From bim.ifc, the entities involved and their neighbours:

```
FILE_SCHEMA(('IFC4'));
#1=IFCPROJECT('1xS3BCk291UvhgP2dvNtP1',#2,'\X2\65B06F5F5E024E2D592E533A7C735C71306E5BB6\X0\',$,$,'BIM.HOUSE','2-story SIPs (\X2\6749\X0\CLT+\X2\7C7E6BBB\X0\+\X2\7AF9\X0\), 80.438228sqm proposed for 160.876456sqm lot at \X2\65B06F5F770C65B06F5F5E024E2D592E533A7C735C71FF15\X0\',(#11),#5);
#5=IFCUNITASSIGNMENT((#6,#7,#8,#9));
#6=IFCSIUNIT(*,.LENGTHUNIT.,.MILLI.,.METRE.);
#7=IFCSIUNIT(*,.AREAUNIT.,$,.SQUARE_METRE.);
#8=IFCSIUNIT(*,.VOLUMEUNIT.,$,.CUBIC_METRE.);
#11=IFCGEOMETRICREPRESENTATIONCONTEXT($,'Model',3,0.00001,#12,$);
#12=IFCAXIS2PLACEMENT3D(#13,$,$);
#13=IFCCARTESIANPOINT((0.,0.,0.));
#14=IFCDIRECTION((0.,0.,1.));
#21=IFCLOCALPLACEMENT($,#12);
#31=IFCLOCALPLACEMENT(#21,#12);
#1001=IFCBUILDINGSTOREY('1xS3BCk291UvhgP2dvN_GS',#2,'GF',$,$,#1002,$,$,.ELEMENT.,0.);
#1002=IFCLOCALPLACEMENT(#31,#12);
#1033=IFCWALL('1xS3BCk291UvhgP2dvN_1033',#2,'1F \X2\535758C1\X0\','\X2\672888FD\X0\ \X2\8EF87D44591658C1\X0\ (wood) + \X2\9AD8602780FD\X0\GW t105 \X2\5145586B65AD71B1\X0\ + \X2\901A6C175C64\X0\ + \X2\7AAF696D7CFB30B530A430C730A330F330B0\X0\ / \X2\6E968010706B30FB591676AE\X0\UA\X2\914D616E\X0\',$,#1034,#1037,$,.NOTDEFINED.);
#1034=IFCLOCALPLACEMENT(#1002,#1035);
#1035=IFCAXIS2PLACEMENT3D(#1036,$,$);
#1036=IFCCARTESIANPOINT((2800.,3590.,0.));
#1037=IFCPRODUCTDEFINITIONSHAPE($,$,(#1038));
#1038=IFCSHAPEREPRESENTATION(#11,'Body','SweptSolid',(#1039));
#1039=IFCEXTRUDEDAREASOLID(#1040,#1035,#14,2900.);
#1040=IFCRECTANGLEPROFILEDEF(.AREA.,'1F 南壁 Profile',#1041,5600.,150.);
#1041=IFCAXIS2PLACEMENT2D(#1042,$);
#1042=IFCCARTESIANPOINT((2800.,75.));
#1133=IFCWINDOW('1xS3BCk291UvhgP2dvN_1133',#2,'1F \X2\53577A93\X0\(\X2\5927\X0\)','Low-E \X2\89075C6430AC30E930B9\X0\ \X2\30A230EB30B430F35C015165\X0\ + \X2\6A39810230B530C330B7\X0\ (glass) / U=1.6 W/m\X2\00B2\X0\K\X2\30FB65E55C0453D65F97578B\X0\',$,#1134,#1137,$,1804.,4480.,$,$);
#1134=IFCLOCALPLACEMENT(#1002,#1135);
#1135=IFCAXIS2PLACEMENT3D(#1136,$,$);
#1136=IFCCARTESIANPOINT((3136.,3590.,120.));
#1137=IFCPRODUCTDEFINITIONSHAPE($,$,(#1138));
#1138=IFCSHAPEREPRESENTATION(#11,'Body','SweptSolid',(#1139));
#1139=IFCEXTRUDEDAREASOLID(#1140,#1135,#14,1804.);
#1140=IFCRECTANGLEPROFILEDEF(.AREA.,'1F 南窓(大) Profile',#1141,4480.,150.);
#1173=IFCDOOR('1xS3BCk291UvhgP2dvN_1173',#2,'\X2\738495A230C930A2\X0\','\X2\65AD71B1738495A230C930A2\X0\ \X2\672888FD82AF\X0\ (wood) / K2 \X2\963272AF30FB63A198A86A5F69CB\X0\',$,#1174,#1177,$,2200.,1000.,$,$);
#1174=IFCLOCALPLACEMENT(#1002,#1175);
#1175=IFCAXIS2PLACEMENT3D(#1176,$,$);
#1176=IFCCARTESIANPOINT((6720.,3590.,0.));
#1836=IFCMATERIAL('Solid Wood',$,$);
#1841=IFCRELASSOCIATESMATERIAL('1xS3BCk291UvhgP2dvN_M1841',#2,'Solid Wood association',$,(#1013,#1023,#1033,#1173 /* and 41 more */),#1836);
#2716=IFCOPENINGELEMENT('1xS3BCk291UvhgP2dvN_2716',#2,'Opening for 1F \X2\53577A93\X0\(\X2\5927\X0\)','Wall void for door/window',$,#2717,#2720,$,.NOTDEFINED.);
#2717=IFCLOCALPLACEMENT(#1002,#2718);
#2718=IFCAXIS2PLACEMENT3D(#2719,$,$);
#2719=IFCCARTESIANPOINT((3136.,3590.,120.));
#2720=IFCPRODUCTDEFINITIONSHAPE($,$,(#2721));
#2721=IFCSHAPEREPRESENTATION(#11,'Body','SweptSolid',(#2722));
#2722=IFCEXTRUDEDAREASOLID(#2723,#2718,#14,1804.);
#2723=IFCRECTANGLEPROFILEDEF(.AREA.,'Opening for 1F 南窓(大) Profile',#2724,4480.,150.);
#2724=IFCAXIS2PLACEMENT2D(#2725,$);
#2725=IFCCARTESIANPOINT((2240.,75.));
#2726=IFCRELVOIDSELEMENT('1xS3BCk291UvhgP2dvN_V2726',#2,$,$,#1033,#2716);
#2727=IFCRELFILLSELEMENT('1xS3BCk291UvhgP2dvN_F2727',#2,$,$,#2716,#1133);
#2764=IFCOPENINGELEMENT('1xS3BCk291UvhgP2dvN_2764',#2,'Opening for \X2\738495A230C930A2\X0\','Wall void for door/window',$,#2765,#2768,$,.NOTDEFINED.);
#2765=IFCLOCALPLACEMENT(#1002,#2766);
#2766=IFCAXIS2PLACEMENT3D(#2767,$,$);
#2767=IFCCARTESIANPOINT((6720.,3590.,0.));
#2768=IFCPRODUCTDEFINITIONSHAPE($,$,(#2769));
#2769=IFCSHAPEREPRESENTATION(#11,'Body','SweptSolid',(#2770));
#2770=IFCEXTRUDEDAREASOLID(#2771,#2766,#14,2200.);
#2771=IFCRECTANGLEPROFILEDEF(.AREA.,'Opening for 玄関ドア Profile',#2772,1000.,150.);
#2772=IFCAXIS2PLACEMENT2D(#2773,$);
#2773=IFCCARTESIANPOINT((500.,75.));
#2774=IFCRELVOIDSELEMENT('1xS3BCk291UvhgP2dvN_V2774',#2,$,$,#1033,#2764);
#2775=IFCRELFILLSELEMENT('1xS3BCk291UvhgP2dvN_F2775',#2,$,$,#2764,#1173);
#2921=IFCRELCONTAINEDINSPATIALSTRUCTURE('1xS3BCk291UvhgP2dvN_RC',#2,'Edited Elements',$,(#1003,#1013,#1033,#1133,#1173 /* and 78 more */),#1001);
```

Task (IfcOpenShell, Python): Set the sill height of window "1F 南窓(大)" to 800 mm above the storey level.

```python
import numpy as np
import ifcopenshell
import ifcopenshell.api.geometry
import ifcopenshell.geom
import ifcopenshell.util.element
import ifcopenshell.util.placement
import ifcopenshell.util.shape
import ifcopenshell.util.unit

model = ifcopenshell.open("bim.ifc")
unit_scale = ifcopenshell.util.unit.calculate_unit_scale(model)

window = model.by_id(1133)
opening = window.FillsVoids[0].RelatingOpeningElement
storey = ifcopenshell.util.element.get_container(window, ifc_class="IfcBuildingStorey")
level = ifcopenshell.util.placement.get_local_placement(storey.ObjectPlacement)[2, 3]

# The opening's origin need not be at the sill, so measure its lowest point.
shape = ifcopenshell.geom.create_shape(ifcopenshell.geom.settings(), opening)
bottom = ifcopenshell.util.shape.get_shape_bottom_elevation(shape, shape.geometry) / unit_scale
dz = level + 0.8 / unit_scale - bottom

shift = np.array([0.0, 0.0, dz])
# The window is not placed relative to its opening, so move both.
for product in (opening, window):
    matrix = ifcopenshell.util.placement.get_local_placement(product.ObjectPlacement)
    matrix[:3, 3] += shift
    ifcopenshell.api.geometry.edit_object_placement(model, product=product, matrix=matrix, is_si=False)

print(f"moved by {dz * unit_scale:+.3f} m")

model.write("bim_edited.ifc")
```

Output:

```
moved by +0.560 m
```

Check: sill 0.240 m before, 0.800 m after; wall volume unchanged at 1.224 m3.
